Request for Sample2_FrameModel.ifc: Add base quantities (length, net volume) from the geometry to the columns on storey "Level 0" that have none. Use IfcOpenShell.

First a look at what the model holds.

```python
import ifcopenshell
import ifcopenshell.util.element
import ifcopenshell.util.unit

model = ifcopenshell.open("Sample2_FrameModel.ifc")
print(model.schema)
for unit_type in ("LENGTHUNIT", "AREAUNIT", "VOLUMEUNIT"):
    print(unit_type, ifcopenshell.util.unit.calculate_unit_scale(model, unit_type))
storey = next(s for s in model.by_type("IfcBuildingStorey") if s.Name == "Level 0")
columns = [e for e in ifcopenshell.util.element.get_decomposition(storey) if e.is_a("IfcColumn")]
for e in sorted(columns, key=lambda e: e.id()):
    print(e.id(), e.is_a(), e.Name, list(ifcopenshell.util.element.get_psets(e, qtos_only=True)), sep=" | ")
```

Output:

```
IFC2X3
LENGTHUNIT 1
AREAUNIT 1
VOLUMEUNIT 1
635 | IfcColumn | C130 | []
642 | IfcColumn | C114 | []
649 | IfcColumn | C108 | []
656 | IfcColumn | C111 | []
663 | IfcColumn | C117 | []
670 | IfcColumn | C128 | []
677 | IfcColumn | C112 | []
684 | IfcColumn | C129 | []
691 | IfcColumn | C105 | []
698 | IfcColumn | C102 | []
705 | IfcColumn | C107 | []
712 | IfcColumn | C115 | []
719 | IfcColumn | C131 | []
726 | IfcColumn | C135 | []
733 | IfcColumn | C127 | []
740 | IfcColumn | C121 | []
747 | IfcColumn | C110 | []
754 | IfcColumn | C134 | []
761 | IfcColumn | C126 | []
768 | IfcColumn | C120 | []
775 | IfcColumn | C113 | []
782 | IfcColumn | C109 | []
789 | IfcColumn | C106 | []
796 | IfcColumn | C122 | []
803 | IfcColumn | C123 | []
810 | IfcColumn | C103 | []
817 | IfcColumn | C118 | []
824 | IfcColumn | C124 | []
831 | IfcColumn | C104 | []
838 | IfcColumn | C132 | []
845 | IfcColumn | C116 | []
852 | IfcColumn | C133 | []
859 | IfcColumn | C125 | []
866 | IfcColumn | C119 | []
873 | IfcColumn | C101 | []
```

```python
import ifcopenshell
import ifcopenshell.api.pset
import ifcopenshell.geom
import ifcopenshell.util.element
import ifcopenshell.util.shape
import ifcopenshell.util.unit

model = ifcopenshell.open("Sample2_FrameModel.ifc")
unit_scale = ifcopenshell.util.unit.calculate_unit_scale(model)
volume_scale = ifcopenshell.util.unit.calculate_unit_scale(model, "VOLUMEUNIT")
settings = ifcopenshell.geom.settings()

storey = next(s for s in model.by_type("IfcBuildingStorey") if s.Name == "Level 0")
columns = [e for e in ifcopenshell.util.element.get_decomposition(storey) if e.is_a("IfcColumn")]

for e in sorted(columns, key=lambda e: e.id()):
    if ifcopenshell.util.element.get_psets(e, qtos_only=True, should_inherit=False):
        continue
    # Geometry comes back in metres, in the element's own axes.
    shape = ifcopenshell.geom.create_shape(settings, e)
    values = {
        "Length": ifcopenshell.util.shape.get_z(shape.geometry) / unit_scale,
        "NetVolume": ifcopenshell.util.shape.get_volume(shape.geometry) / volume_scale,
    }
    qto = ifcopenshell.api.pset.add_qto(model, product=e, name="BaseQuantities")
    ifcopenshell.api.pset.edit_qto(model, qto=qto, properties=values)
    print(e.id(), {k: round(v, 3) for k, v in values.items()})

model.write("Sample2_FrameModel_edited.ifc")
```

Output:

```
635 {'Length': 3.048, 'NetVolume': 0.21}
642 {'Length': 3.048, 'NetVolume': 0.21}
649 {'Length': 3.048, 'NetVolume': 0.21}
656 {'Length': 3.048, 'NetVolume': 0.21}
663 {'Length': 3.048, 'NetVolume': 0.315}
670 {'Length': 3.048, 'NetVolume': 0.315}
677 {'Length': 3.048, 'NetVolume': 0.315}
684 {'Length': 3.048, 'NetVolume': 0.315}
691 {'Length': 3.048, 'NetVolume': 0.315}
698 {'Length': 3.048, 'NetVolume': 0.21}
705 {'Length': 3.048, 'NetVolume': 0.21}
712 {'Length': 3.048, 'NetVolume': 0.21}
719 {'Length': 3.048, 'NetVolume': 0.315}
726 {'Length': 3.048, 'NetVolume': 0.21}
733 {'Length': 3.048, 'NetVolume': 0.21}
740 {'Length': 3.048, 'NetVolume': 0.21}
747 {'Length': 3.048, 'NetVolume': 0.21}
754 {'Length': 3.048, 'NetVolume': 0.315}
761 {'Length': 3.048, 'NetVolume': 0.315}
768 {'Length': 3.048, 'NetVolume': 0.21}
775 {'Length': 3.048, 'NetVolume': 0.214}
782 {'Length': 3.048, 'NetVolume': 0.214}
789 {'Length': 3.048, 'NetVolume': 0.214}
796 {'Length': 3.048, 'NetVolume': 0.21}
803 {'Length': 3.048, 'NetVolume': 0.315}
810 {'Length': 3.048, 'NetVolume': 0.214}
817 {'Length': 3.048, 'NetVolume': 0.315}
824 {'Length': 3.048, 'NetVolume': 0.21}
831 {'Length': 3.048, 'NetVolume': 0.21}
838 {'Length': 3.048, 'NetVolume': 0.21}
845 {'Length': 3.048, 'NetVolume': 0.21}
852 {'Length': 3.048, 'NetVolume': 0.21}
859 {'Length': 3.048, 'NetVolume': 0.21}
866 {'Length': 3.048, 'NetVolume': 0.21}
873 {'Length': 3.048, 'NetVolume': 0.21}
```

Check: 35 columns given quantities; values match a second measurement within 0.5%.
